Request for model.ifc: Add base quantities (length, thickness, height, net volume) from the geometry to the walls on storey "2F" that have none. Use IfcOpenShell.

First a look at what the model holds.

```python
import ifcopenshell
import ifcopenshell.util.element
import ifcopenshell.util.unit

model = ifcopenshell.open("model.ifc")
print(model.schema)
for unit_type in ("LENGTHUNIT", "AREAUNIT", "VOLUMEUNIT"):
    print(unit_type, ifcopenshell.util.unit.calculate_unit_scale(model, unit_type))
storey = next(s for s in model.by_type("IfcBuildingStorey") if s.Name == "2F")
walls = [e for e in ifcopenshell.util.element.get_decomposition(storey) if e.is_a("IfcWall")]
for e in sorted(walls, key=lambda e: e.id()):
    print(e.id(), e.is_a(), e.Name, list(ifcopenshell.util.element.get_psets(e, qtos_only=True)), sep=" | ")
```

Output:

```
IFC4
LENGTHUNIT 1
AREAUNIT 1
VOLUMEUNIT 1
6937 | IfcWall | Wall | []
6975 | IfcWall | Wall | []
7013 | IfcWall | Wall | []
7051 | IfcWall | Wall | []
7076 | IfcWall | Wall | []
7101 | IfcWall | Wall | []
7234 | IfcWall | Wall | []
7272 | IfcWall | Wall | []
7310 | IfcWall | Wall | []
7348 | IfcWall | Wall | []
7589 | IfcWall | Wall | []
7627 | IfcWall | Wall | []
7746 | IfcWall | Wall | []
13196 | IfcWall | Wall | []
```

```python
import ifcopenshell
import ifcopenshell.api.pset
import ifcopenshell.geom
import ifcopenshell.util.element
import ifcopenshell.util.shape
import ifcopenshell.util.unit

model = ifcopenshell.open("model.ifc")
unit_scale = ifcopenshell.util.unit.calculate_unit_scale(model)
volume_scale = ifcopenshell.util.unit.calculate_unit_scale(model, "VOLUMEUNIT")
settings = ifcopenshell.geom.settings()

storey = next(s for s in model.by_type("IfcBuildingStorey") if s.Name == "2F")
walls = [e for e in ifcopenshell.util.element.get_decomposition(storey) if e.is_a("IfcWall")]

for e in sorted(walls, key=lambda e: e.id()):
    if ifcopenshell.util.element.get_psets(e, qtos_only=True, should_inherit=False):
        continue
    # Geometry comes back in metres, in the element's own axes.
    shape = ifcopenshell.geom.create_shape(settings, e)
    values = {
        "Length": ifcopenshell.util.shape.get_x(shape.geometry) / unit_scale,
        "Width": ifcopenshell.util.shape.get_y(shape.geometry) / unit_scale,
        "Height": ifcopenshell.util.shape.get_z(shape.geometry) / unit_scale,
        "NetVolume": ifcopenshell.util.shape.get_volume(shape.geometry) / volume_scale,
    }
    qto = ifcopenshell.api.pset.add_qto(model, product=e, name="Qto_WallBaseQuantities")
    ifcopenshell.api.pset.edit_qto(model, qto=qto, properties=values)
    print(e.id(), {k: round(v, 3) for k, v in values.items()})

model.write("model_rev.ifc")
```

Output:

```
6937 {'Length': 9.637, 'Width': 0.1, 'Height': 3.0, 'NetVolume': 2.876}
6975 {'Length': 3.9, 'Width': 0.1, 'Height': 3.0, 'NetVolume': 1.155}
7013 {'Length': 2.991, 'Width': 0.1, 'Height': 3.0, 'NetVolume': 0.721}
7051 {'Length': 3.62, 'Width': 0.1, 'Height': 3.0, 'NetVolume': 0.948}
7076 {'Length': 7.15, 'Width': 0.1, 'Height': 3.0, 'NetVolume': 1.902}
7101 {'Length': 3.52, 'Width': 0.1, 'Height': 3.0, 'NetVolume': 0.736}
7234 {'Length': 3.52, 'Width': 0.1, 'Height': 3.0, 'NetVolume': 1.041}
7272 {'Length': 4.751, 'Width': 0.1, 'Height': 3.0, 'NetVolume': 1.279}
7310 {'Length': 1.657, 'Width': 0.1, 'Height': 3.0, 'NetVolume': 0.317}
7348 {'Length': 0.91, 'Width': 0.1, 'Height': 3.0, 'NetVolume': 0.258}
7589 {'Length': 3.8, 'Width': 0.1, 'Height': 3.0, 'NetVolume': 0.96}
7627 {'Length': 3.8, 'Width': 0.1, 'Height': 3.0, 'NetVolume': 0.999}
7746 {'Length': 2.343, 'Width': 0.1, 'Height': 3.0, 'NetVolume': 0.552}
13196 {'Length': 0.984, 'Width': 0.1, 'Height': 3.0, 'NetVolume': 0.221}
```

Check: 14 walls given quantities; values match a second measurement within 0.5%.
